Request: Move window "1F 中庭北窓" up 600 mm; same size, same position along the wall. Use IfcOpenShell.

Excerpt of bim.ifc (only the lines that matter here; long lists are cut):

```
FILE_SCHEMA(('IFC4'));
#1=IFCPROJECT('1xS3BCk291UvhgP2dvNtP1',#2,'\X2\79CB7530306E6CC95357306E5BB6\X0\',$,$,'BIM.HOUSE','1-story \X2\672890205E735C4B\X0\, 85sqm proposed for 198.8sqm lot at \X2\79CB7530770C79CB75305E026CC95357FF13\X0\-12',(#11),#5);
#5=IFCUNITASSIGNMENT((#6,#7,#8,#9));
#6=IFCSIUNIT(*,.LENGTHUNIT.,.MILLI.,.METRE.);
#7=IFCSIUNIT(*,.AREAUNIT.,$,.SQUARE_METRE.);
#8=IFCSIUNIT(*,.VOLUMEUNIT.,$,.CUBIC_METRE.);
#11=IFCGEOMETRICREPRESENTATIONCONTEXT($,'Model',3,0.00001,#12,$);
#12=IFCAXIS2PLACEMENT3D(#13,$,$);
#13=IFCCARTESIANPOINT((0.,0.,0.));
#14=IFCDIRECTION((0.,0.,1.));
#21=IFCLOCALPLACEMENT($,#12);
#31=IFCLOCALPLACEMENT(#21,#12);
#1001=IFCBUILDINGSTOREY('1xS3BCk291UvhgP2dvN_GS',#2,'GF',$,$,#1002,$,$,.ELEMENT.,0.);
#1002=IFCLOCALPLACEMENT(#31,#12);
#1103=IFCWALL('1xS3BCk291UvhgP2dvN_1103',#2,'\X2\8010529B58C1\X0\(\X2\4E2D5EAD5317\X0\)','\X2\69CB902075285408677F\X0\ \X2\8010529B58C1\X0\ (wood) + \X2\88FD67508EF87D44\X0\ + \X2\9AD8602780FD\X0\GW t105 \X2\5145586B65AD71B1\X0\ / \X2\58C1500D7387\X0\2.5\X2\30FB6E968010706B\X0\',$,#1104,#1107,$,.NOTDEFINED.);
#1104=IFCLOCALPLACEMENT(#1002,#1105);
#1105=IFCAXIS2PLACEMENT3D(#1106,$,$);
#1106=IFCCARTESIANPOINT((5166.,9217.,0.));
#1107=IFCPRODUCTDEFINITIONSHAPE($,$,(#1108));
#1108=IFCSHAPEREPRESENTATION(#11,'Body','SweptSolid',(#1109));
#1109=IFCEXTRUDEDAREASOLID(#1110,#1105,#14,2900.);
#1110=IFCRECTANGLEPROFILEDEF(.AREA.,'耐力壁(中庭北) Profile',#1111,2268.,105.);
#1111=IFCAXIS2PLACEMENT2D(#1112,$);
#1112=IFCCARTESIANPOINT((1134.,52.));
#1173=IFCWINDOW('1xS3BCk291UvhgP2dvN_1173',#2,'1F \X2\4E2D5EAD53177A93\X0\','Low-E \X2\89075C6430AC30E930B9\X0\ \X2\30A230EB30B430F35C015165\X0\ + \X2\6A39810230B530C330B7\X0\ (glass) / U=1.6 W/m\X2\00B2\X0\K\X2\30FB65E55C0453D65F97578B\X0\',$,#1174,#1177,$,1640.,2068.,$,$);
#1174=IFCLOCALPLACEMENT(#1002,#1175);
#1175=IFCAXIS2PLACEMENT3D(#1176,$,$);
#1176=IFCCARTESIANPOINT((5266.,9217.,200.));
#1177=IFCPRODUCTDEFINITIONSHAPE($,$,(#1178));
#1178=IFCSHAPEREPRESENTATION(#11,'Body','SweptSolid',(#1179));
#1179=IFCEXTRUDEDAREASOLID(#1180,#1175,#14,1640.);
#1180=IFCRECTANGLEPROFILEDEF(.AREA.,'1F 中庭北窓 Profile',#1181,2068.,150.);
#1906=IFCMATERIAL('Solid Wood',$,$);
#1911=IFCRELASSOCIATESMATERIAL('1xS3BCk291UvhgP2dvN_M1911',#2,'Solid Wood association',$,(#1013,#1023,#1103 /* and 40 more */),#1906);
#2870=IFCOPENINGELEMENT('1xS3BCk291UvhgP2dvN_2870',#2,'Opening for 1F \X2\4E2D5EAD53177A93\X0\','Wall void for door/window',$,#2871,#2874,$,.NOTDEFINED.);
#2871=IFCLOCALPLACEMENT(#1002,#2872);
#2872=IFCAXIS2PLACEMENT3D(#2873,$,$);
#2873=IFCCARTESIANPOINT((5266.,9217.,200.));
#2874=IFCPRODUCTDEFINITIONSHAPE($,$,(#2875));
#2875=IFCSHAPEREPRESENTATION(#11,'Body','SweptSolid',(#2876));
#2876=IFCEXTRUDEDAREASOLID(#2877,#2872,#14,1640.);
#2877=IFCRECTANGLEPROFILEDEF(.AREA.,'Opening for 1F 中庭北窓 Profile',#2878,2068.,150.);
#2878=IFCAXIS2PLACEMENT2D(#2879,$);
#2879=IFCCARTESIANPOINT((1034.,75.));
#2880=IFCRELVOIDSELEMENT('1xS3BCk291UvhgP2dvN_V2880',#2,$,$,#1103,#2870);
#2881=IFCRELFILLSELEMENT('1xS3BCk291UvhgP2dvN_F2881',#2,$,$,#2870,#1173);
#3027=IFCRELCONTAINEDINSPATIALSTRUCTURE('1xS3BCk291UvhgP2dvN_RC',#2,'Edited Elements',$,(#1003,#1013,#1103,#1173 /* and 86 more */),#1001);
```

```python
import numpy as np
import ifcopenshell
import ifcopenshell.api.geometry
import ifcopenshell.util.placement
import ifcopenshell.util.unit

model = ifcopenshell.open("bim.ifc")
unit_scale = ifcopenshell.util.unit.calculate_unit_scale(model)

window = model.by_guid("1xS3BCk291UvhgP2dvN_1173")
opening = window.FillsVoids[0].RelatingOpeningElement
dz = 0.6 / unit_scale

shift = np.array([0.0, 0.0, dz])
# The window is not placed relative to its opening, so move both.
for product in (opening, window):
    matrix = ifcopenshell.util.placement.get_local_placement(product.ObjectPlacement)
    matrix[:3, 3] += shift
    ifcopenshell.api.geometry.edit_object_placement(model, product=product, matrix=matrix, is_si=False)

print(f"moved by {dz * unit_scale:+.3f} m")

model.write("bim-out.ifc")
```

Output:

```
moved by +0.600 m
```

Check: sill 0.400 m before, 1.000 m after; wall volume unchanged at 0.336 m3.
